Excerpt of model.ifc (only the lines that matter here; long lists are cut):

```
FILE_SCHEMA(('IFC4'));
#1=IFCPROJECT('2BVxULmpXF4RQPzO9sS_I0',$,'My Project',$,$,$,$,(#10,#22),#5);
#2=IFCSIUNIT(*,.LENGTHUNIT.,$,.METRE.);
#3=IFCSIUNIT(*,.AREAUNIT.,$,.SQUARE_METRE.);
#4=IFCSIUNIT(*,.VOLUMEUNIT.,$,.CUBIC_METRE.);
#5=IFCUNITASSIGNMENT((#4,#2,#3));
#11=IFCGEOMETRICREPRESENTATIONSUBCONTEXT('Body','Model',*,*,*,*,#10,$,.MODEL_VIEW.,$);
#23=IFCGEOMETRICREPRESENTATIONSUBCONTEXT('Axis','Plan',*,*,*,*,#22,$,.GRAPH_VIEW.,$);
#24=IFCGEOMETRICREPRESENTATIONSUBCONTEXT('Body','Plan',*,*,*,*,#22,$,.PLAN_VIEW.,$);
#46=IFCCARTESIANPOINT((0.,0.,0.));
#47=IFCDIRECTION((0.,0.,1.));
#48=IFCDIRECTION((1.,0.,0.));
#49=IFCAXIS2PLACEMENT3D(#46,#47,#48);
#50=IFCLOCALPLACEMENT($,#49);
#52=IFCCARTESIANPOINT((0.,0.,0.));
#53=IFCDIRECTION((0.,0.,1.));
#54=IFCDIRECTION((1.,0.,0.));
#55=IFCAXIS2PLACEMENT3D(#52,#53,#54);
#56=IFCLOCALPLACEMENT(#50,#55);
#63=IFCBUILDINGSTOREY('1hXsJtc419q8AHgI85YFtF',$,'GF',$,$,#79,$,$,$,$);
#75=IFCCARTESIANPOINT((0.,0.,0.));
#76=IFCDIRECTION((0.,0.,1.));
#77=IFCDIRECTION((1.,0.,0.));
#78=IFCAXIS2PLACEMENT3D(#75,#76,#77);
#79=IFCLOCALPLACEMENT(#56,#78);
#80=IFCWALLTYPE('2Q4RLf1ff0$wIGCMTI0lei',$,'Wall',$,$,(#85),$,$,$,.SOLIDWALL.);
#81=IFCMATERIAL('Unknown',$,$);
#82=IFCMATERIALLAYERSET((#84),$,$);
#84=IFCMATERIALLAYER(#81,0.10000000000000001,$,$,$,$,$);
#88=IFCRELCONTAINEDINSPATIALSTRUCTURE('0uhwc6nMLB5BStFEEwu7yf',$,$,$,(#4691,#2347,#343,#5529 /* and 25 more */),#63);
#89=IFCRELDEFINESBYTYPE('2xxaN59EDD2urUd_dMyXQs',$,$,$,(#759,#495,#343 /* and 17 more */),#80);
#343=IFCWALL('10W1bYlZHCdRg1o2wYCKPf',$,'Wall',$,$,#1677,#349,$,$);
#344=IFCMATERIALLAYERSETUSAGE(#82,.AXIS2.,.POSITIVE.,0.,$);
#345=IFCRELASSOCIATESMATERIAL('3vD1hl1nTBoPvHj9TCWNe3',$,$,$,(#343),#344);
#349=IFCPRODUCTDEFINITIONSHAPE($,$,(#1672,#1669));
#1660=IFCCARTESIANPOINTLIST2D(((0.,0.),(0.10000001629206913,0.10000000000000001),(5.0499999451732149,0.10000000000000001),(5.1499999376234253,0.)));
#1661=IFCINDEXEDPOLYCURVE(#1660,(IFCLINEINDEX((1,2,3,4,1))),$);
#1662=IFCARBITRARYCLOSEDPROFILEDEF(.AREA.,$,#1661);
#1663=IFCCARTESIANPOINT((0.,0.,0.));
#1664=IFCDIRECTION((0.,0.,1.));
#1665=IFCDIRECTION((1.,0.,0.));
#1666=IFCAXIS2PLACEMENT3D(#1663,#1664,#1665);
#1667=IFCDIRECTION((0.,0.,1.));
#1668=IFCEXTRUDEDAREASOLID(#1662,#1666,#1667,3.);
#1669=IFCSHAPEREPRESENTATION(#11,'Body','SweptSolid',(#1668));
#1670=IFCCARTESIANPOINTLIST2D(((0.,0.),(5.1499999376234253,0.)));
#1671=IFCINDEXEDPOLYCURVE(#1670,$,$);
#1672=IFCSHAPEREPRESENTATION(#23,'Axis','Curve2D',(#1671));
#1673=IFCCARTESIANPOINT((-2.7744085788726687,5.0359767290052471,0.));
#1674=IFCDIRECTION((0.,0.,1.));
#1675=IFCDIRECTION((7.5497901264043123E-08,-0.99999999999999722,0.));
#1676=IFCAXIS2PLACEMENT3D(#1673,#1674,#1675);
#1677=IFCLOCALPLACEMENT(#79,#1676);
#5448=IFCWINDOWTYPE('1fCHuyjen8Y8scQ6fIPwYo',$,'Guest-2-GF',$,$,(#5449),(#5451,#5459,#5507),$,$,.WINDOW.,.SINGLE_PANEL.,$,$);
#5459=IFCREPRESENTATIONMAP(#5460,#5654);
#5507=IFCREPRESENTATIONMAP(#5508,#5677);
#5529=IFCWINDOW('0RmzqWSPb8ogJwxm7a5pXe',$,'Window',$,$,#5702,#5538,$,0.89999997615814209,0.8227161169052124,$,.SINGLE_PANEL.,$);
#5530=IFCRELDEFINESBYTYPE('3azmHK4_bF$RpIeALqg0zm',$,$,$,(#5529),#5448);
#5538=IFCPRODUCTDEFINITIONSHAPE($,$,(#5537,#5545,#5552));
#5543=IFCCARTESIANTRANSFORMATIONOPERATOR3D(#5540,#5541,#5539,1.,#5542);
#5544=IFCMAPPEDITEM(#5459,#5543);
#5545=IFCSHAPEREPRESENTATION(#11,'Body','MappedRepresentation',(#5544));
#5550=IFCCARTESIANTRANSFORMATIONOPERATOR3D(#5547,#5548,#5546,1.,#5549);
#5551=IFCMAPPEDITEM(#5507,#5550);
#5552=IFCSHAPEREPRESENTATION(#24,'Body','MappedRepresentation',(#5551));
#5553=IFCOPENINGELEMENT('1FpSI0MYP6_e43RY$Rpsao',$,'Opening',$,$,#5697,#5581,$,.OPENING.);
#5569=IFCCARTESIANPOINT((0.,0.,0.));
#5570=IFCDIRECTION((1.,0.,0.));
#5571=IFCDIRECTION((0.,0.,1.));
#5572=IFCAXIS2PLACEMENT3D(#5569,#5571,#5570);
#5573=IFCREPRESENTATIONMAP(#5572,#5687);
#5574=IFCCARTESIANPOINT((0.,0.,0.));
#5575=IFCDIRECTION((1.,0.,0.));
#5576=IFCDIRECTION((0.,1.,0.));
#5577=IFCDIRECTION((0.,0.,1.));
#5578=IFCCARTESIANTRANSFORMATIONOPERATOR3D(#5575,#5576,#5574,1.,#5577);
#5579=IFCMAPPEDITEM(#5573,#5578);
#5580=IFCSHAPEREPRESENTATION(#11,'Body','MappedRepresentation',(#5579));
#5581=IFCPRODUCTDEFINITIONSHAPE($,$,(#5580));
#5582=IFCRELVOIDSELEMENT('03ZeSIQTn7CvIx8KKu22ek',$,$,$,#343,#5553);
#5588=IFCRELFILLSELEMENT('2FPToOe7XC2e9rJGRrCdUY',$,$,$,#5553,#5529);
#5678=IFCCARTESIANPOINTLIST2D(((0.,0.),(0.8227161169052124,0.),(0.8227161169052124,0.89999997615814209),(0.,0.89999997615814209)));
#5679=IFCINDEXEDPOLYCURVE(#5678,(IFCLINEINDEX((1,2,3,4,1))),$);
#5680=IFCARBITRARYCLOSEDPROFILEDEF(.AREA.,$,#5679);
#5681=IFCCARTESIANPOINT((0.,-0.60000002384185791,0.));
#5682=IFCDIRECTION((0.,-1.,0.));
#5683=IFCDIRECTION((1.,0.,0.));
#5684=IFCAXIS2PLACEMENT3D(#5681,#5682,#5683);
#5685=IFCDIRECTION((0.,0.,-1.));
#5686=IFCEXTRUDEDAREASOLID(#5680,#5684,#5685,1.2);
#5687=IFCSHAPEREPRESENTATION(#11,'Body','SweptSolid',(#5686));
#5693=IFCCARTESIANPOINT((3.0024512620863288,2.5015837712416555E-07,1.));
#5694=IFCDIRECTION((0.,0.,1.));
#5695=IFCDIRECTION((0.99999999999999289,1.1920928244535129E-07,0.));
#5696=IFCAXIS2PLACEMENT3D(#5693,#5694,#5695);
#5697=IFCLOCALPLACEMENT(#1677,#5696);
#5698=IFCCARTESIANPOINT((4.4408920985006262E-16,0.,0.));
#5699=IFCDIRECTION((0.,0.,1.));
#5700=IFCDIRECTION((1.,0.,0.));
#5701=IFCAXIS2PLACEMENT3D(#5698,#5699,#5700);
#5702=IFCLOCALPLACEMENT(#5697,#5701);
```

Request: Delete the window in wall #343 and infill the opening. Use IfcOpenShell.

```python
import ifcopenshell
import ifcopenshell.api.feature
import ifcopenshell.api.root
import ifcopenshell.geom
import ifcopenshell.util.shape

model = ifcopenshell.open("model.ifc")
settings = ifcopenshell.geom.settings()


def volume(element):
    """Net volume in cubic metres, openings subtracted."""
    shape = ifcopenshell.geom.create_shape(settings, element)
    return ifcopenshell.util.shape.get_volume(shape.geometry)


window = model.by_guid("0RmzqWSPb8ogJwxm7a5pXe")
opening = window.FillsVoids[0].RelatingOpeningElement
wall = opening.VoidsElements[0].RelatingBuildingElement
before = volume(wall)

ifcopenshell.api.root.remove_product(model, product=window)
ifcopenshell.api.feature.remove_feature(model, feature=opening)

after = volume(wall)

print(f"wall volume {before:.3f} -> {after:.3f} m3")

model.write("model_edited.ifc")
```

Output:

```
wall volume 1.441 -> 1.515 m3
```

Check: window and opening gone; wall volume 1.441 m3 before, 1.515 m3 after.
